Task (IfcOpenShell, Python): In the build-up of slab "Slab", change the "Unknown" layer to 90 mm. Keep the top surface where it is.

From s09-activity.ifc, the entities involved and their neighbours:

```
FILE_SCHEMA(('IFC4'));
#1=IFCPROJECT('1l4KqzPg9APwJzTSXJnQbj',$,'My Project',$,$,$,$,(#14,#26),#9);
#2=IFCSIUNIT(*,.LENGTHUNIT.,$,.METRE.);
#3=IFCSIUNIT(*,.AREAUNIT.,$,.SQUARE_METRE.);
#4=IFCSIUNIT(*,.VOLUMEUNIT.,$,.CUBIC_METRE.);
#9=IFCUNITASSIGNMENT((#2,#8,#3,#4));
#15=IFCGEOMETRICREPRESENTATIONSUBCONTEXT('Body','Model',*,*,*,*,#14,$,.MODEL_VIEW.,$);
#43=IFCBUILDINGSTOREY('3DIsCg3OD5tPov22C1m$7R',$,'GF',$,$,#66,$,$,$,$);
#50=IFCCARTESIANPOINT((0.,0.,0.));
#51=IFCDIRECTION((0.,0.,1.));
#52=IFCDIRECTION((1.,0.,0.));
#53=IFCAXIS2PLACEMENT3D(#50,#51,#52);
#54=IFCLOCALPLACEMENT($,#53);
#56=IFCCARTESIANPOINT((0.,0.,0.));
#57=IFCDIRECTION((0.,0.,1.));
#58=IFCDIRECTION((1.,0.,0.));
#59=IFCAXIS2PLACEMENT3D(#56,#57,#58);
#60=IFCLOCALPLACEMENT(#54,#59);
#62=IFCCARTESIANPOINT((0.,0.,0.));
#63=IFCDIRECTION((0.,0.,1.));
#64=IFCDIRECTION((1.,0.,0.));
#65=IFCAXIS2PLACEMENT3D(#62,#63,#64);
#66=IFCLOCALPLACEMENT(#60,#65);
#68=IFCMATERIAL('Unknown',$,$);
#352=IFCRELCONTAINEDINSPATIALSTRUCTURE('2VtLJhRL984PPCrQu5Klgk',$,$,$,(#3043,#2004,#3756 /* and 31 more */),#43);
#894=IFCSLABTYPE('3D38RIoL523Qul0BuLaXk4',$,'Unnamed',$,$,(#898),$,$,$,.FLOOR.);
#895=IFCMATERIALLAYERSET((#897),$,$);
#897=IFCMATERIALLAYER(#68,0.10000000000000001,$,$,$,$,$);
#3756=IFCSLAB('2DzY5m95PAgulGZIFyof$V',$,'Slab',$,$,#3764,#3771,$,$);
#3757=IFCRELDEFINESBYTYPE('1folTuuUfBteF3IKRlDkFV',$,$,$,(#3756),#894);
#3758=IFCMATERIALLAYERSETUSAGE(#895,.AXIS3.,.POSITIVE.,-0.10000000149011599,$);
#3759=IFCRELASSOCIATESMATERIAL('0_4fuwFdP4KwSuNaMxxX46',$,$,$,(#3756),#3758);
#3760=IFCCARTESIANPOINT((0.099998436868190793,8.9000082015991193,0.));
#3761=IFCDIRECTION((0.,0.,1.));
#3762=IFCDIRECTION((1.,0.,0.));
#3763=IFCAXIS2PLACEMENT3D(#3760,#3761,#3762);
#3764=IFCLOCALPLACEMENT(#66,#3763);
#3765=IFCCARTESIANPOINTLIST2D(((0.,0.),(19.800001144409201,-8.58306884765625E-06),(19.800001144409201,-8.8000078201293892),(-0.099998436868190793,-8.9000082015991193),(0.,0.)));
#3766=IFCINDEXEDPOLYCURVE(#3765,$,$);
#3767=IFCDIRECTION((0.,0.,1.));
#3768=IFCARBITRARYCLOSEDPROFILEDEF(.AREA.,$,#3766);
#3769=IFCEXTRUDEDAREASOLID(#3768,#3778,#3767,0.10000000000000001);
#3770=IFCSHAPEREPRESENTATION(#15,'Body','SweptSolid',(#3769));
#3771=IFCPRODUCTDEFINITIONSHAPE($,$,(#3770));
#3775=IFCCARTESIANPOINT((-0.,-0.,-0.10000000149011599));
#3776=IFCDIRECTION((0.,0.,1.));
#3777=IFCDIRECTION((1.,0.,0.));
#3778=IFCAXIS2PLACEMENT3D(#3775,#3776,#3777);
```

```python
import ifcopenshell
import ifcopenshell.util.element
import ifcopenshell.util.representation
import ifcopenshell.util.unit

model = ifcopenshell.open("s09-activity.ifc")
unit_scale = ifcopenshell.util.unit.calculate_unit_scale(model)

layer_set = model.by_id(895)
layer = next(l for l in layer_set.MaterialLayers if l.Material and l.Material.Name == "Unknown")
change = 0.09 / unit_scale - layer.LayerThickness
layer.LayerThickness += change

# Geometry does not follow the layer set by itself.
slabs = [e for e in ifcopenshell.util.element.get_elements_by_material(model, layer_set) if e.is_a("IfcSlab")]
for slab in sorted(slabs, key=lambda e: e.id()):
    body = ifcopenshell.util.representation.get_representation(slab, "Model", "Body")
    solid = body.Items[0]
    old_depth = solid.Depth
    solid.Depth += change
    # Extruded upwards: lower the start of the extrusion so the top stays.
    x, y, z = solid.Position.Location.Coordinates
    solid.Position.Location = model.createIfcCartesianPoint((x, y, z - change))
    print(slab.id(), f"{old_depth:g} -> {solid.Depth:g}")

# The layers are counted up from the underside, which has moved.
for usage in {ifcopenshell.util.element.get_material(slab) for slab in slabs}:
    usage.OffsetFromReferenceLine -= change

model.write("s09-activity_rev.ifc")
```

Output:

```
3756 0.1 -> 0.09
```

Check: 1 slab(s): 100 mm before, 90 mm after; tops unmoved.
